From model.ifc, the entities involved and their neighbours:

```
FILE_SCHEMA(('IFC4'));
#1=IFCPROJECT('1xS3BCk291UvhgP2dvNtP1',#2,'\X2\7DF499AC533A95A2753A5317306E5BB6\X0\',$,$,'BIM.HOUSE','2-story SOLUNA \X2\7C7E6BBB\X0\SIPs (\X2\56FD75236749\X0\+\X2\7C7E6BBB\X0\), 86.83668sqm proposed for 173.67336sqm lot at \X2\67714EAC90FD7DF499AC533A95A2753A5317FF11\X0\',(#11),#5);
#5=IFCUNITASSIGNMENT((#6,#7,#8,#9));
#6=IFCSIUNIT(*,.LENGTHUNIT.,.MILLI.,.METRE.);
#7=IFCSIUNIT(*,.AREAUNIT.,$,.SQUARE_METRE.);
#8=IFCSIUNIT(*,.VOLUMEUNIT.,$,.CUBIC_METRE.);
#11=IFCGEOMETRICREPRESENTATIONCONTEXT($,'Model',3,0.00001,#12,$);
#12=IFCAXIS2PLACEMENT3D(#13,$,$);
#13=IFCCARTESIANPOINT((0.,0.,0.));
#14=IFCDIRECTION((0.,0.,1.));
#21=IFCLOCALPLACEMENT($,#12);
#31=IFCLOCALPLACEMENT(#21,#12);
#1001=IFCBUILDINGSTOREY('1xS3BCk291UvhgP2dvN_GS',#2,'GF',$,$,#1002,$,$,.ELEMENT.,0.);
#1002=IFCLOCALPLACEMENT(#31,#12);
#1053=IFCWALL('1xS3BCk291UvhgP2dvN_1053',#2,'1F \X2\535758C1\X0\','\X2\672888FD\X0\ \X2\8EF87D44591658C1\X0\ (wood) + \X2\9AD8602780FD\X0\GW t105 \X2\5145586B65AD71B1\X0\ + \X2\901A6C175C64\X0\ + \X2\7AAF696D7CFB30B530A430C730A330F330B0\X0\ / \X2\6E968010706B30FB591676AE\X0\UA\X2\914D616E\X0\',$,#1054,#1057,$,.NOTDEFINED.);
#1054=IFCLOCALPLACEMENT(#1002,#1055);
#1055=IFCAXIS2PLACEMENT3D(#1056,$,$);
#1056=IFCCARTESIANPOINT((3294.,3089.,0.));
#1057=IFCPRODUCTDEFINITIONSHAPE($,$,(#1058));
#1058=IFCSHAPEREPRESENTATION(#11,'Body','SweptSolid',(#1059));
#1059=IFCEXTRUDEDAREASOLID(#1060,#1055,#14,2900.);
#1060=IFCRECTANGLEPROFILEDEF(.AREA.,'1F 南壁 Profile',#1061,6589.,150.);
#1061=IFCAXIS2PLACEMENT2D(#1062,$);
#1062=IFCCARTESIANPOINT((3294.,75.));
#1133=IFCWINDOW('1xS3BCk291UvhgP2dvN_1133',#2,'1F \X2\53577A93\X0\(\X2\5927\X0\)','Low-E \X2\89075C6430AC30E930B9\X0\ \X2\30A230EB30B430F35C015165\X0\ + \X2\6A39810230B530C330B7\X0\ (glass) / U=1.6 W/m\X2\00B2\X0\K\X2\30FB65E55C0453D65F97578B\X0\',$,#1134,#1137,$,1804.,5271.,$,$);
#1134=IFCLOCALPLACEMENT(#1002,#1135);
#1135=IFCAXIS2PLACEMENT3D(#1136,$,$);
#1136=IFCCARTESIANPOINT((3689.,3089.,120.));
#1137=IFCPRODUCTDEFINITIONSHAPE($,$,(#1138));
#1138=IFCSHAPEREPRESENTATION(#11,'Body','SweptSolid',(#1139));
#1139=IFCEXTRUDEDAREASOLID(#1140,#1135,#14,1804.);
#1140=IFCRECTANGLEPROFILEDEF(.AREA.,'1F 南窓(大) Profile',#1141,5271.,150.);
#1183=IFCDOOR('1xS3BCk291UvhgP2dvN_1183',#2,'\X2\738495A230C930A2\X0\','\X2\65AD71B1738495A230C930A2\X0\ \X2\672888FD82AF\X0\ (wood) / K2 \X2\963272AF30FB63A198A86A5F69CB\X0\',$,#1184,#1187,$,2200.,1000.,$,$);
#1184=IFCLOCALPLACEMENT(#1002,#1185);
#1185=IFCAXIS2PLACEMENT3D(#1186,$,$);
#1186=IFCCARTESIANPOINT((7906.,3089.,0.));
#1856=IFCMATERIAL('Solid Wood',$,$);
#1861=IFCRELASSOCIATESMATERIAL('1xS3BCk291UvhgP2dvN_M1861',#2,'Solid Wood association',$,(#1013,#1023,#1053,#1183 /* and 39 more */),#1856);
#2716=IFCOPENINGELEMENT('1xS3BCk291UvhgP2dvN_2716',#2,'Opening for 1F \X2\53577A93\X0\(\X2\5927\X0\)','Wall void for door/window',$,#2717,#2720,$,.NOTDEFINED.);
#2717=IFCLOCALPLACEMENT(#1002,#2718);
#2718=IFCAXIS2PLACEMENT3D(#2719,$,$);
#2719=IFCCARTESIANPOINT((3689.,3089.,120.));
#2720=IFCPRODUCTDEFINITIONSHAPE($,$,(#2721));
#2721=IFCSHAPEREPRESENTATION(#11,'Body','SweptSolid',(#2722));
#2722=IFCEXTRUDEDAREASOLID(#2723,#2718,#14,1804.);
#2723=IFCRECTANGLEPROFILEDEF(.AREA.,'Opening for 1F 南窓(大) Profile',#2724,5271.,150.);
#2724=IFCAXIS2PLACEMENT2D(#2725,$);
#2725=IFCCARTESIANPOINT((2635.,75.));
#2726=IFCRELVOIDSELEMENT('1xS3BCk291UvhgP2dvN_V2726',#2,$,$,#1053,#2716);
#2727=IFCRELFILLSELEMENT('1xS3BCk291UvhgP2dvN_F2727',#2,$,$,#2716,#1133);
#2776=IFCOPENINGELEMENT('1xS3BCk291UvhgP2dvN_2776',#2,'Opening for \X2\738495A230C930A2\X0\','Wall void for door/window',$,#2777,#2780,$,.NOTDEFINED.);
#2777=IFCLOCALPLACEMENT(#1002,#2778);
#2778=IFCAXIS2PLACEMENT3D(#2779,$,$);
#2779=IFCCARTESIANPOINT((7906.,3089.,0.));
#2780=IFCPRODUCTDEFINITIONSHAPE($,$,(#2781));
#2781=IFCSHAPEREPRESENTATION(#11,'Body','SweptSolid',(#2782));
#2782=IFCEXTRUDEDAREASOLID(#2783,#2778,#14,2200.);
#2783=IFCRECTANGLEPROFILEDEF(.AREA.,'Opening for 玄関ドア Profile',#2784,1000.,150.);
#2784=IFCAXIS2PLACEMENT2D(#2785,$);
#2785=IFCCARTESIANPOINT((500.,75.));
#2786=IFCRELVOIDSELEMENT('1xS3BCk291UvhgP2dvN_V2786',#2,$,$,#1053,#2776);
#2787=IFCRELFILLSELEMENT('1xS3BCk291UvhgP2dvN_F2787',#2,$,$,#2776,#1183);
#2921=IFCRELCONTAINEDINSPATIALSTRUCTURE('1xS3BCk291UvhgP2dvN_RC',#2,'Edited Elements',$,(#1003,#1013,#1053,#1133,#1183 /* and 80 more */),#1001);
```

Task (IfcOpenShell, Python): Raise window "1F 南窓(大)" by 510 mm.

```python
import numpy as np
import ifcopenshell
import ifcopenshell.api.geometry
import ifcopenshell.util.placement
import ifcopenshell.util.unit

model = ifcopenshell.open("model.ifc")
unit_scale = ifcopenshell.util.unit.calculate_unit_scale(model)

window = model.by_guid("1xS3BCk291UvhgP2dvN_1133")
opening = window.FillsVoids[0].RelatingOpeningElement
dz = 0.51 / unit_scale

shift = np.array([0.0, 0.0, dz])
# The window is not placed relative to its opening, so move both.
for product in (opening, window):
    matrix = ifcopenshell.util.placement.get_local_placement(product.ObjectPlacement)
    matrix[:3, 3] += shift
    ifcopenshell.api.geometry.edit_object_placement(model, product=product, matrix=matrix, is_si=False)

print(f"moved by {dz * unit_scale:+.3f} m")

model.write("model_v2.ifc")
```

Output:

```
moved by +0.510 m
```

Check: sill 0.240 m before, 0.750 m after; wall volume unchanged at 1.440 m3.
